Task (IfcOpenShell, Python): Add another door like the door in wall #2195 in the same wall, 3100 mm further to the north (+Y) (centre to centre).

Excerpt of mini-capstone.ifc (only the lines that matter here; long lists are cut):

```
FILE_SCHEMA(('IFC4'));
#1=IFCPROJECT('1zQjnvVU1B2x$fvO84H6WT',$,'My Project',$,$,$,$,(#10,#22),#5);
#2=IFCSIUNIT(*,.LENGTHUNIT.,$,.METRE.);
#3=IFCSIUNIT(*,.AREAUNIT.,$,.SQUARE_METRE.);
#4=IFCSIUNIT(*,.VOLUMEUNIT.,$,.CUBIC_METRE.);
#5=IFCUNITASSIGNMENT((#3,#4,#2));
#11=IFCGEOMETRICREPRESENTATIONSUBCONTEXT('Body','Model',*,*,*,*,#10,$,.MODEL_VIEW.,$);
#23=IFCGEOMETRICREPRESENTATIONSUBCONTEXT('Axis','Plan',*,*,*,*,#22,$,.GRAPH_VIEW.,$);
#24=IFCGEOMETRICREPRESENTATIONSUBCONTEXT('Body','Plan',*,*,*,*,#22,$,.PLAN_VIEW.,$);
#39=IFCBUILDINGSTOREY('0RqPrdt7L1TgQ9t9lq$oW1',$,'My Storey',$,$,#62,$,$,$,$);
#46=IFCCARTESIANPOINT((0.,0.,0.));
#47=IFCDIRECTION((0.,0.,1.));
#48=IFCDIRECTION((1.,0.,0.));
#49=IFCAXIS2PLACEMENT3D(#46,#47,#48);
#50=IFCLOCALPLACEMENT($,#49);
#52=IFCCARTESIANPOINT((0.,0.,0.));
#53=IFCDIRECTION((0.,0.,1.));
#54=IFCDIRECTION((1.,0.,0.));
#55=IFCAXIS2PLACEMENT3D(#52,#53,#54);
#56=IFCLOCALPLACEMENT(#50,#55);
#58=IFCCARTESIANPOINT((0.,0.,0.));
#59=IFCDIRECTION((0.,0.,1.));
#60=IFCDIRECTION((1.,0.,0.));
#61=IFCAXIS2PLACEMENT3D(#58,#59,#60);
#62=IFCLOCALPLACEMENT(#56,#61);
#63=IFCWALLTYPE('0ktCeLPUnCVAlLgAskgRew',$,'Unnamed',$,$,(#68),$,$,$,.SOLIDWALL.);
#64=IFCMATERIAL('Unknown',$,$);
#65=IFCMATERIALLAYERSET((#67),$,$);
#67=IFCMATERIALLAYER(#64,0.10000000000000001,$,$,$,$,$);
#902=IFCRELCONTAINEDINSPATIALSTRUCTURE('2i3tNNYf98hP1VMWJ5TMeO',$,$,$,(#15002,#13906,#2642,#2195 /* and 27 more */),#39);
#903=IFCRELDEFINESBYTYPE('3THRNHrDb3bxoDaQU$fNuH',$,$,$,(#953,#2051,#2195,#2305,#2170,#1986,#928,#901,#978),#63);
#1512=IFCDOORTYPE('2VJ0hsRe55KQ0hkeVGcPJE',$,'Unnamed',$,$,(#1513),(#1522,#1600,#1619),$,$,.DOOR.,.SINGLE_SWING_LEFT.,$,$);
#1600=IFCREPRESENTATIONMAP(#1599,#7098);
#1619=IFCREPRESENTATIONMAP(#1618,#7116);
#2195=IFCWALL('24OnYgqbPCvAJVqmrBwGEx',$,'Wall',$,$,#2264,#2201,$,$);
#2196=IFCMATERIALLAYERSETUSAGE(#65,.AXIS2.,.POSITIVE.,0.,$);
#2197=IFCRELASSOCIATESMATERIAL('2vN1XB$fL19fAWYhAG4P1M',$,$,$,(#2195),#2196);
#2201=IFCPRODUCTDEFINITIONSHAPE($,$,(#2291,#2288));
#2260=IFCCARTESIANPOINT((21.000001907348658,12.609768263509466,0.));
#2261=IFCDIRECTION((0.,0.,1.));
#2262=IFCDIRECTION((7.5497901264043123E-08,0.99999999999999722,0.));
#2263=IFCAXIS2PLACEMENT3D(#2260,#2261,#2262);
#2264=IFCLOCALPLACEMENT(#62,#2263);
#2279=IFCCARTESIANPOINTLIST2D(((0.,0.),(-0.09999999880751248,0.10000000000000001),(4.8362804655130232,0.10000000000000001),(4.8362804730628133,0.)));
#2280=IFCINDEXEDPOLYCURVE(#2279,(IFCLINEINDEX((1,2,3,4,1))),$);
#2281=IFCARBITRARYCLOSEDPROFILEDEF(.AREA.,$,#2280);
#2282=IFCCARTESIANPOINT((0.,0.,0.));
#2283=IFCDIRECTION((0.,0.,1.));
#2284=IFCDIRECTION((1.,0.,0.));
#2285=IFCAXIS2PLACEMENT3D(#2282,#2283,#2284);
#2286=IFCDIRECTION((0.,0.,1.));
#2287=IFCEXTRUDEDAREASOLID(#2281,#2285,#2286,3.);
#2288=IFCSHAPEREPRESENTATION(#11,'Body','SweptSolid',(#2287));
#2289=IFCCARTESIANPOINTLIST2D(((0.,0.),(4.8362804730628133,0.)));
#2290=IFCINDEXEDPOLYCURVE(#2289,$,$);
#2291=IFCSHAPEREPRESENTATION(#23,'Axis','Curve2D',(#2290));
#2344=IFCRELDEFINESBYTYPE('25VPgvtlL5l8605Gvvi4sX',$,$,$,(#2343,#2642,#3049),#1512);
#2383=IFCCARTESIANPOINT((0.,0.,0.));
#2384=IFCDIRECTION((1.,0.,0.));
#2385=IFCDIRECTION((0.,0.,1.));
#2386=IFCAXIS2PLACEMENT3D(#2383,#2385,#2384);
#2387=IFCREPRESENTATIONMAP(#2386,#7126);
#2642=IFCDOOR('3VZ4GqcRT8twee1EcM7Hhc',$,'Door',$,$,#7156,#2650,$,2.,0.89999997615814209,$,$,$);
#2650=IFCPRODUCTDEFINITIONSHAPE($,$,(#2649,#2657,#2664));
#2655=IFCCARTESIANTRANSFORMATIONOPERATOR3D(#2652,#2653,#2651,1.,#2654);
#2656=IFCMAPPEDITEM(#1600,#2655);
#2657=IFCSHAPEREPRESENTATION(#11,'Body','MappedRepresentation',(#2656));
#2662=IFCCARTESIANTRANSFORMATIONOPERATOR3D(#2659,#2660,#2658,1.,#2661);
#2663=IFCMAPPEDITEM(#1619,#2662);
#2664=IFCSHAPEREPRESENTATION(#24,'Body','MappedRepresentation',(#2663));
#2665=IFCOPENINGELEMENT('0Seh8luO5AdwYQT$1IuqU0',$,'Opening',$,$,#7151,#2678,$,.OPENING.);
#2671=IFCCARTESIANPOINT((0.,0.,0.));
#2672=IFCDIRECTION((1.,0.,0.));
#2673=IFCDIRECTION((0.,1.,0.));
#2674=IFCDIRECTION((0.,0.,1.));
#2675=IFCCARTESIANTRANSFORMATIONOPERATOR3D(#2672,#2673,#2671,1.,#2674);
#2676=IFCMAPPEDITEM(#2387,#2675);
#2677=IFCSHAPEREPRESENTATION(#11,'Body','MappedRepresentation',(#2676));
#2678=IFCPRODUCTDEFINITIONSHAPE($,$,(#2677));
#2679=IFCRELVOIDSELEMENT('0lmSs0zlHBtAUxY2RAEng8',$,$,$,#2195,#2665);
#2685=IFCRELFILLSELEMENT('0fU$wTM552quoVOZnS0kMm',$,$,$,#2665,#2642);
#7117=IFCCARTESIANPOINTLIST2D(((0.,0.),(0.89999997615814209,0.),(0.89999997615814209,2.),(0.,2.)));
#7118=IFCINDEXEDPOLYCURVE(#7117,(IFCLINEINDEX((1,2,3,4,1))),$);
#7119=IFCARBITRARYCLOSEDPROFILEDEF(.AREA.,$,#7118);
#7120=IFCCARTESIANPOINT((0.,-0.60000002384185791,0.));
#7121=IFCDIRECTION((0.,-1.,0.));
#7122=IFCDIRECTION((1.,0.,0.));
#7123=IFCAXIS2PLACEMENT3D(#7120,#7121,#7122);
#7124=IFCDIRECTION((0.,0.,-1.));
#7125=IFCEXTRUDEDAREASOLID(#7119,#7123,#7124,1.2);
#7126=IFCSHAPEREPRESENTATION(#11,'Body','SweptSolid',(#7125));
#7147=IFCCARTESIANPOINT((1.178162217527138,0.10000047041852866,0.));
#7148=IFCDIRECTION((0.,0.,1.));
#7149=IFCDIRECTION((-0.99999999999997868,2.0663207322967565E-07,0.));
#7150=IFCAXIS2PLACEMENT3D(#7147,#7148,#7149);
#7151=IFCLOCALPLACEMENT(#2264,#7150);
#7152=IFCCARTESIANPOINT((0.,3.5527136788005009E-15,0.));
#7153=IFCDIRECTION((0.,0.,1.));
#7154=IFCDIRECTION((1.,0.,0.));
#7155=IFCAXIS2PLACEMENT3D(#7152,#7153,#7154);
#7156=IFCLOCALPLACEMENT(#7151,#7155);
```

```python
import ifcopenshell
import ifcopenshell.api.feature
import ifcopenshell.api.geometry
import ifcopenshell.api.root
import ifcopenshell.geom
import ifcopenshell.util.element
import ifcopenshell.util.placement
import ifcopenshell.util.shape

model = ifcopenshell.open("mini-capstone.ifc")
settings = ifcopenshell.geom.settings()


def volume(element):
    """Net volume in cubic metres, openings subtracted."""
    shape = ifcopenshell.geom.create_shape(settings, element)
    return ifcopenshell.util.shape.get_volume(shape.geometry)


door = model.by_guid("3VZ4GqcRT8twee1EcM7Hhc")
opening = door.FillsVoids[0].RelatingOpeningElement
wall = opening.VoidsElements[0].RelatingBuildingElement
before = volume(wall)
shift = ifcopenshell.util.placement.get_local_placement(wall.ObjectPlacement)[:3, 0] * 3.1

# copy_class copies the void relationship, type, container and properties, but no geometry.
new_opening = ifcopenshell.api.root.copy_class(model, product=opening)
new_opening.Representation = ifcopenshell.util.element.copy_deep(
    model, opening.Representation, exclude=["IfcGeometricRepresentationContext", "IfcRepresentationMap"]
)
new_door = ifcopenshell.api.root.copy_class(model, product=door)
new_door.Representation = ifcopenshell.util.element.copy_deep(
    model, door.Representation, exclude=["IfcGeometricRepresentationContext", "IfcRepresentationMap"]
)
ifcopenshell.api.feature.add_filling(model, opening=new_opening, element=new_door)

for old, new in ((opening, new_opening), (door, new_door)):
    matrix = ifcopenshell.util.placement.get_local_placement(old.ObjectPlacement)
    matrix[:3, 3] += shift
    ifcopenshell.api.geometry.edit_object_placement(model, product=new, matrix=matrix, is_si=False)

after = volume(wall)

print(f"wall volume {before:.3f} -> {after:.3f} m3")

model.write("mini-capstone_updated.ifc")
```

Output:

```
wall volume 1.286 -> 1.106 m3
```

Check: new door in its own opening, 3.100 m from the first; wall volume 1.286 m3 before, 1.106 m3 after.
